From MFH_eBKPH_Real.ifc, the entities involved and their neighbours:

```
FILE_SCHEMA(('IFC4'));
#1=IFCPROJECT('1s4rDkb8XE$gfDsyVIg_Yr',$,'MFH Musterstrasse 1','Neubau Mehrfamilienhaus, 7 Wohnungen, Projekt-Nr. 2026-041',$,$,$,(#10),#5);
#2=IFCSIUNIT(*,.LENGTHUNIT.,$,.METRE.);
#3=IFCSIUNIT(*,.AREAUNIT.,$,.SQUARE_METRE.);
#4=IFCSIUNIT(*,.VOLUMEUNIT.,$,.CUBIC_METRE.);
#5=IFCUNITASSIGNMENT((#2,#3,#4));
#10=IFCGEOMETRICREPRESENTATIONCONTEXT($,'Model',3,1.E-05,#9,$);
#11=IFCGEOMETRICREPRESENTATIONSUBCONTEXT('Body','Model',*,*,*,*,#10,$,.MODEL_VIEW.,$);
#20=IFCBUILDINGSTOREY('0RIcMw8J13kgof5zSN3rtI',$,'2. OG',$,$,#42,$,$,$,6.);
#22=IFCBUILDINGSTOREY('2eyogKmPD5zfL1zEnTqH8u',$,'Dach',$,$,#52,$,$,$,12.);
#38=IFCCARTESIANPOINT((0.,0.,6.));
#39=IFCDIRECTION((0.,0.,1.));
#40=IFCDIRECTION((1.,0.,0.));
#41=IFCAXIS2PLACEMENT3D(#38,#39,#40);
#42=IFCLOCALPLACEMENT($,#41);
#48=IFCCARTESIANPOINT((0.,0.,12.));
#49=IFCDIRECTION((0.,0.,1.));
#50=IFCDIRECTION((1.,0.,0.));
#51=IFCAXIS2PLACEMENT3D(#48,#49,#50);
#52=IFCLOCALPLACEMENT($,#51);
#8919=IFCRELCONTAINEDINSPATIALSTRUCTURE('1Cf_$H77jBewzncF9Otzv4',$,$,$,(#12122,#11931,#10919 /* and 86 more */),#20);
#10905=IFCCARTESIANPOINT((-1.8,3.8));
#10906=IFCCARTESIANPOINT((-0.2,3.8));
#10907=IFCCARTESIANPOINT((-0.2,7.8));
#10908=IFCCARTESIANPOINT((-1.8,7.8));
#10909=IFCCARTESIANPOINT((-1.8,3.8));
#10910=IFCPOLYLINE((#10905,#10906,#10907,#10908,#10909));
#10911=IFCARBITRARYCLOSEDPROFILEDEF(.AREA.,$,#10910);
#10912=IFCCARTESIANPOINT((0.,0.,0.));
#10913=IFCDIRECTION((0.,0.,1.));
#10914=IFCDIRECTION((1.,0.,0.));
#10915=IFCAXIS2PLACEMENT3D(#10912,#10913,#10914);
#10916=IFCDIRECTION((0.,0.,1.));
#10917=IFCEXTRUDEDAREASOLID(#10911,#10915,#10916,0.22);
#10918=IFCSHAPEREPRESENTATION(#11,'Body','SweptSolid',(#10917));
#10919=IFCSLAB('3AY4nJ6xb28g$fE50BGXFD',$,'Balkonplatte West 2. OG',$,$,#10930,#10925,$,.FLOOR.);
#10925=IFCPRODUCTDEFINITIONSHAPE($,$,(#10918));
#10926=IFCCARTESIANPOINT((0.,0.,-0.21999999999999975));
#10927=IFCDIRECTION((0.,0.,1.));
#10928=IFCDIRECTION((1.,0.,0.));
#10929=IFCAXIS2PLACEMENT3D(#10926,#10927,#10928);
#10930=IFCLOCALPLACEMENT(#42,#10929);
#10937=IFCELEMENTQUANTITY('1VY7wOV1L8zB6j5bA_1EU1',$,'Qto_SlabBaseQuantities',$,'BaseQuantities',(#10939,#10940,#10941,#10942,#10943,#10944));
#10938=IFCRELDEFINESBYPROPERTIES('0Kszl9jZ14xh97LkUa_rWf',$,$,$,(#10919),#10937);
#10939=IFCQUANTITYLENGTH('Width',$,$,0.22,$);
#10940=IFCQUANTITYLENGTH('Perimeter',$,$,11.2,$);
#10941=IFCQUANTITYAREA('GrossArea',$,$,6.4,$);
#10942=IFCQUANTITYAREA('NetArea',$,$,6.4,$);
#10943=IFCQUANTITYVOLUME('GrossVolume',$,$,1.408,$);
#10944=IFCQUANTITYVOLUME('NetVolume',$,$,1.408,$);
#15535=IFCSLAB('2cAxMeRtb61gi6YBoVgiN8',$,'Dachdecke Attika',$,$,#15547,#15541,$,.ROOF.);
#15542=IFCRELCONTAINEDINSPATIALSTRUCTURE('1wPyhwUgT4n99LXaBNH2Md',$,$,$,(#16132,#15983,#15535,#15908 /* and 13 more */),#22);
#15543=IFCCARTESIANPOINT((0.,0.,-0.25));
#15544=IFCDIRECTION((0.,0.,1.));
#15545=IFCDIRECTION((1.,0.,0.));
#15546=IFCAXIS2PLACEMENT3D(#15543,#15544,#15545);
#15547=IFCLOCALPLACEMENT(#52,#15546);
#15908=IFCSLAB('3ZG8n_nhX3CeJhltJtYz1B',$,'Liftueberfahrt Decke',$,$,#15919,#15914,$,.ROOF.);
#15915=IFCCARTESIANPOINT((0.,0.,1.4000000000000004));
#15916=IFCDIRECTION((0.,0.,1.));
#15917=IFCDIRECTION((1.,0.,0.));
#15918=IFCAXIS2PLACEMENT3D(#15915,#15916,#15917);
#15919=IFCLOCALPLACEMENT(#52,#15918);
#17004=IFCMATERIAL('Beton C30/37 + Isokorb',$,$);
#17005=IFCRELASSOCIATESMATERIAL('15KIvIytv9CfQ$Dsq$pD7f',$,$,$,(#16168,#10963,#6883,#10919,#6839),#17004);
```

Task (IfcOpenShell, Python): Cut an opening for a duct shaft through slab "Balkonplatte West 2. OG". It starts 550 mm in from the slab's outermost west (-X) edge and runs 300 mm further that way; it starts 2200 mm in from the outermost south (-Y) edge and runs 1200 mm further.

```python
import numpy as np
import ifcopenshell
import ifcopenshell.api.feature
import ifcopenshell.api.geometry
import ifcopenshell.api.pset
import ifcopenshell.api.root
import ifcopenshell.geom
import ifcopenshell.util.element
import ifcopenshell.util.placement
import ifcopenshell.util.representation
import ifcopenshell.util.shape
import ifcopenshell.util.unit

model = ifcopenshell.open("MFH_eBKPH_Real.ifc")
unit_scale = ifcopenshell.util.unit.calculate_unit_scale(model)
area_scale = ifcopenshell.util.unit.calculate_unit_scale(model, "AREAUNIT")
volume_scale = ifcopenshell.util.unit.calculate_unit_scale(model, "VOLUMEUNIT")
settings = ifcopenshell.geom.settings()


def volume(element):
    """Net volume in cubic metres, openings subtracted."""
    shape = ifcopenshell.geom.create_shape(settings, element)
    return ifcopenshell.util.shape.get_volume(shape.geometry)


slab = model.by_id(10919)
before = volume(slab)

# Extent in the slab's own axes, in metres. The edges named are its -X and -Y sides.
slab_shape = ifcopenshell.geom.create_shape(settings, slab)
vertices = ifcopenshell.util.shape.get_vertices(slab_shape.geometry)
x_min, y_min, bottom = vertices.min(axis=0)
top = vertices[:, 2].max()

opening = ifcopenshell.api.root.create_entity(model, ifc_class="IfcOpeningElement", name="Duct shaft opening", predefined_type="OPENING")
context = ifcopenshell.util.representation.get_context(model, "Model", "Body", "MODEL_VIEW")
width, depth = 0.3, 1.2
outline = [(0.0, 0.0), (width, 0.0), (width, depth), (0.0, depth), (0.0, 0.0)]
# Overshoot both faces by 50 mm so the cut is clean.
shape = ifcopenshell.api.geometry.add_slab_representation(
    model, context=context, depth=top - bottom + 0.1, polyline=outline
)
ifcopenshell.api.geometry.assign_representation(model, product=opening, representation=shape)

matrix = ifcopenshell.util.placement.get_local_placement(slab.ObjectPlacement)
matrix[:, 3] = matrix @ np.append(np.array([x_min + 0.55, y_min + 2.2, bottom - 0.05]) / unit_scale, 1.0)
ifcopenshell.api.geometry.edit_object_placement(model, product=opening, matrix=matrix, is_si=False)
ifcopenshell.api.feature.add_feature(model, feature=opening, element=slab)

after = volume(slab)

# Update the slab's stored quantities.
qto = model.by_id(ifcopenshell.util.element.get_pset(slab, "Qto_SlabBaseQuantities", should_inherit=False)["id"])
ifcopenshell.api.pset.edit_qto(model, qto=qto, properties={
    "NetArea": after / (top - bottom) / area_scale,
    "NetVolume": after / volume_scale,
})

print(f"slab volume {before:.3f} -> {after:.3f} m3")

model.write("MFH_eBKPH_Real_updated.ifc")
```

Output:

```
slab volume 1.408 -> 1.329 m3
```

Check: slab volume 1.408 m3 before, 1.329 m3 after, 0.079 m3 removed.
